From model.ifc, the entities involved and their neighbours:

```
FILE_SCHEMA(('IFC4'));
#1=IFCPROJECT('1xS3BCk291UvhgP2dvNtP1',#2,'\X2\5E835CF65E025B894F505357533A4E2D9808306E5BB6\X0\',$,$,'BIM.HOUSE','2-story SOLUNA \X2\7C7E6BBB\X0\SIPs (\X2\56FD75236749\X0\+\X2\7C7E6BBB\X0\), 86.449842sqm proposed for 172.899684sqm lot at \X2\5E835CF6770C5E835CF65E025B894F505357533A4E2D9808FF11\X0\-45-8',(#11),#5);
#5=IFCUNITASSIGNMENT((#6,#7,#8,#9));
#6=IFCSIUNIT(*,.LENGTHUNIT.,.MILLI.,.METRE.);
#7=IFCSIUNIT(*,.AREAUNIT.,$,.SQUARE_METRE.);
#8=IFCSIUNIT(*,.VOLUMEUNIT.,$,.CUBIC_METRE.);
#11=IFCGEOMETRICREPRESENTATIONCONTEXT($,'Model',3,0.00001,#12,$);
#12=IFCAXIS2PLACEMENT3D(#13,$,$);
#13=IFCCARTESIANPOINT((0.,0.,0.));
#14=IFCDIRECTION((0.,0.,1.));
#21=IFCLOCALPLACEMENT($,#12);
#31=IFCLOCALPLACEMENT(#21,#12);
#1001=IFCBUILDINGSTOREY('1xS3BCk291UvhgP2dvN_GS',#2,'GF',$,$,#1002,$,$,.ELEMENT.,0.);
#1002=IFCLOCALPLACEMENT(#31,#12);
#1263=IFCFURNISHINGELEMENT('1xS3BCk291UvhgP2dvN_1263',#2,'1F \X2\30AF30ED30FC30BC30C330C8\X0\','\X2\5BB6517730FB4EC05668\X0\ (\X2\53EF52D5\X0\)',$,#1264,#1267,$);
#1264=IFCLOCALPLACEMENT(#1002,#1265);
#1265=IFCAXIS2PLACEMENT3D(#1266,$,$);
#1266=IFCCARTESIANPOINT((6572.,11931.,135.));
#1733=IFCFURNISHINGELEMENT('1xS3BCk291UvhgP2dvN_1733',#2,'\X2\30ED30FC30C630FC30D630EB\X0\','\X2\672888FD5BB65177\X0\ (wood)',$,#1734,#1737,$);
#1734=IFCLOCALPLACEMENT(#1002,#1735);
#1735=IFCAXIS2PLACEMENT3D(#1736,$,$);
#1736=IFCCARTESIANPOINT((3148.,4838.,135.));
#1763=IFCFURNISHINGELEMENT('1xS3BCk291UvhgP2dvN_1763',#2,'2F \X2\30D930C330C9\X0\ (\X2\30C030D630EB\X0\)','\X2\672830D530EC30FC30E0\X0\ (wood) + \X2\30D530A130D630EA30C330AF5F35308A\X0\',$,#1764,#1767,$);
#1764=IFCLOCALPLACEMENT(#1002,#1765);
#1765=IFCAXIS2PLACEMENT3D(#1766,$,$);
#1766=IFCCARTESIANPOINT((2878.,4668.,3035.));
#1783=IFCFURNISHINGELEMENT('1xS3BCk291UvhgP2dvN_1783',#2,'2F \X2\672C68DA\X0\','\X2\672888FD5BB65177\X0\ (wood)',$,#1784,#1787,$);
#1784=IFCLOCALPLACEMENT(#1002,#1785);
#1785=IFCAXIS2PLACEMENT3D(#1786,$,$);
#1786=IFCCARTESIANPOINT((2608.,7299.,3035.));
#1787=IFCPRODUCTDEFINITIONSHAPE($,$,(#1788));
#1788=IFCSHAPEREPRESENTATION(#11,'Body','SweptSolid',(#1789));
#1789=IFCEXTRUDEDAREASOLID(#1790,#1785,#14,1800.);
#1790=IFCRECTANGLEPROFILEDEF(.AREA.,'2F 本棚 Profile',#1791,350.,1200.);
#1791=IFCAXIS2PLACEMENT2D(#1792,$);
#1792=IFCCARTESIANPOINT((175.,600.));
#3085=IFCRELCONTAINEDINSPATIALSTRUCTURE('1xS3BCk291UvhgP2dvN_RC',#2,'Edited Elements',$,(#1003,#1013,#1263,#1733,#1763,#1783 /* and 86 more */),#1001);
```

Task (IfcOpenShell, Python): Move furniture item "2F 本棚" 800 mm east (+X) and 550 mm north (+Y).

```python
import ifcopenshell
import ifcopenshell.api.geometry
import ifcopenshell.util.placement

model = ifcopenshell.open("model.ifc")

item = model.by_guid("1xS3BCk291UvhgP2dvN_1783")
matrix = ifcopenshell.util.placement.get_local_placement(item.ObjectPlacement)
matrix[0, 3] += 800.0
matrix[1, 3] += 550.0
ifcopenshell.api.geometry.edit_object_placement(model, product=item, matrix=matrix, is_si=False)

print(ifcopenshell.util.placement.get_local_placement(item.ObjectPlacement).round(3) + 0.0)

model.write("model_edited.ifc")
```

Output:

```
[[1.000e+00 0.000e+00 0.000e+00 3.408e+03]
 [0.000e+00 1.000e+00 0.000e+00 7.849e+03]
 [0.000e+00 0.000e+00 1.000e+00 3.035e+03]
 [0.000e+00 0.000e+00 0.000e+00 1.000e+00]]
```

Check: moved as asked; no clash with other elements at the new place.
